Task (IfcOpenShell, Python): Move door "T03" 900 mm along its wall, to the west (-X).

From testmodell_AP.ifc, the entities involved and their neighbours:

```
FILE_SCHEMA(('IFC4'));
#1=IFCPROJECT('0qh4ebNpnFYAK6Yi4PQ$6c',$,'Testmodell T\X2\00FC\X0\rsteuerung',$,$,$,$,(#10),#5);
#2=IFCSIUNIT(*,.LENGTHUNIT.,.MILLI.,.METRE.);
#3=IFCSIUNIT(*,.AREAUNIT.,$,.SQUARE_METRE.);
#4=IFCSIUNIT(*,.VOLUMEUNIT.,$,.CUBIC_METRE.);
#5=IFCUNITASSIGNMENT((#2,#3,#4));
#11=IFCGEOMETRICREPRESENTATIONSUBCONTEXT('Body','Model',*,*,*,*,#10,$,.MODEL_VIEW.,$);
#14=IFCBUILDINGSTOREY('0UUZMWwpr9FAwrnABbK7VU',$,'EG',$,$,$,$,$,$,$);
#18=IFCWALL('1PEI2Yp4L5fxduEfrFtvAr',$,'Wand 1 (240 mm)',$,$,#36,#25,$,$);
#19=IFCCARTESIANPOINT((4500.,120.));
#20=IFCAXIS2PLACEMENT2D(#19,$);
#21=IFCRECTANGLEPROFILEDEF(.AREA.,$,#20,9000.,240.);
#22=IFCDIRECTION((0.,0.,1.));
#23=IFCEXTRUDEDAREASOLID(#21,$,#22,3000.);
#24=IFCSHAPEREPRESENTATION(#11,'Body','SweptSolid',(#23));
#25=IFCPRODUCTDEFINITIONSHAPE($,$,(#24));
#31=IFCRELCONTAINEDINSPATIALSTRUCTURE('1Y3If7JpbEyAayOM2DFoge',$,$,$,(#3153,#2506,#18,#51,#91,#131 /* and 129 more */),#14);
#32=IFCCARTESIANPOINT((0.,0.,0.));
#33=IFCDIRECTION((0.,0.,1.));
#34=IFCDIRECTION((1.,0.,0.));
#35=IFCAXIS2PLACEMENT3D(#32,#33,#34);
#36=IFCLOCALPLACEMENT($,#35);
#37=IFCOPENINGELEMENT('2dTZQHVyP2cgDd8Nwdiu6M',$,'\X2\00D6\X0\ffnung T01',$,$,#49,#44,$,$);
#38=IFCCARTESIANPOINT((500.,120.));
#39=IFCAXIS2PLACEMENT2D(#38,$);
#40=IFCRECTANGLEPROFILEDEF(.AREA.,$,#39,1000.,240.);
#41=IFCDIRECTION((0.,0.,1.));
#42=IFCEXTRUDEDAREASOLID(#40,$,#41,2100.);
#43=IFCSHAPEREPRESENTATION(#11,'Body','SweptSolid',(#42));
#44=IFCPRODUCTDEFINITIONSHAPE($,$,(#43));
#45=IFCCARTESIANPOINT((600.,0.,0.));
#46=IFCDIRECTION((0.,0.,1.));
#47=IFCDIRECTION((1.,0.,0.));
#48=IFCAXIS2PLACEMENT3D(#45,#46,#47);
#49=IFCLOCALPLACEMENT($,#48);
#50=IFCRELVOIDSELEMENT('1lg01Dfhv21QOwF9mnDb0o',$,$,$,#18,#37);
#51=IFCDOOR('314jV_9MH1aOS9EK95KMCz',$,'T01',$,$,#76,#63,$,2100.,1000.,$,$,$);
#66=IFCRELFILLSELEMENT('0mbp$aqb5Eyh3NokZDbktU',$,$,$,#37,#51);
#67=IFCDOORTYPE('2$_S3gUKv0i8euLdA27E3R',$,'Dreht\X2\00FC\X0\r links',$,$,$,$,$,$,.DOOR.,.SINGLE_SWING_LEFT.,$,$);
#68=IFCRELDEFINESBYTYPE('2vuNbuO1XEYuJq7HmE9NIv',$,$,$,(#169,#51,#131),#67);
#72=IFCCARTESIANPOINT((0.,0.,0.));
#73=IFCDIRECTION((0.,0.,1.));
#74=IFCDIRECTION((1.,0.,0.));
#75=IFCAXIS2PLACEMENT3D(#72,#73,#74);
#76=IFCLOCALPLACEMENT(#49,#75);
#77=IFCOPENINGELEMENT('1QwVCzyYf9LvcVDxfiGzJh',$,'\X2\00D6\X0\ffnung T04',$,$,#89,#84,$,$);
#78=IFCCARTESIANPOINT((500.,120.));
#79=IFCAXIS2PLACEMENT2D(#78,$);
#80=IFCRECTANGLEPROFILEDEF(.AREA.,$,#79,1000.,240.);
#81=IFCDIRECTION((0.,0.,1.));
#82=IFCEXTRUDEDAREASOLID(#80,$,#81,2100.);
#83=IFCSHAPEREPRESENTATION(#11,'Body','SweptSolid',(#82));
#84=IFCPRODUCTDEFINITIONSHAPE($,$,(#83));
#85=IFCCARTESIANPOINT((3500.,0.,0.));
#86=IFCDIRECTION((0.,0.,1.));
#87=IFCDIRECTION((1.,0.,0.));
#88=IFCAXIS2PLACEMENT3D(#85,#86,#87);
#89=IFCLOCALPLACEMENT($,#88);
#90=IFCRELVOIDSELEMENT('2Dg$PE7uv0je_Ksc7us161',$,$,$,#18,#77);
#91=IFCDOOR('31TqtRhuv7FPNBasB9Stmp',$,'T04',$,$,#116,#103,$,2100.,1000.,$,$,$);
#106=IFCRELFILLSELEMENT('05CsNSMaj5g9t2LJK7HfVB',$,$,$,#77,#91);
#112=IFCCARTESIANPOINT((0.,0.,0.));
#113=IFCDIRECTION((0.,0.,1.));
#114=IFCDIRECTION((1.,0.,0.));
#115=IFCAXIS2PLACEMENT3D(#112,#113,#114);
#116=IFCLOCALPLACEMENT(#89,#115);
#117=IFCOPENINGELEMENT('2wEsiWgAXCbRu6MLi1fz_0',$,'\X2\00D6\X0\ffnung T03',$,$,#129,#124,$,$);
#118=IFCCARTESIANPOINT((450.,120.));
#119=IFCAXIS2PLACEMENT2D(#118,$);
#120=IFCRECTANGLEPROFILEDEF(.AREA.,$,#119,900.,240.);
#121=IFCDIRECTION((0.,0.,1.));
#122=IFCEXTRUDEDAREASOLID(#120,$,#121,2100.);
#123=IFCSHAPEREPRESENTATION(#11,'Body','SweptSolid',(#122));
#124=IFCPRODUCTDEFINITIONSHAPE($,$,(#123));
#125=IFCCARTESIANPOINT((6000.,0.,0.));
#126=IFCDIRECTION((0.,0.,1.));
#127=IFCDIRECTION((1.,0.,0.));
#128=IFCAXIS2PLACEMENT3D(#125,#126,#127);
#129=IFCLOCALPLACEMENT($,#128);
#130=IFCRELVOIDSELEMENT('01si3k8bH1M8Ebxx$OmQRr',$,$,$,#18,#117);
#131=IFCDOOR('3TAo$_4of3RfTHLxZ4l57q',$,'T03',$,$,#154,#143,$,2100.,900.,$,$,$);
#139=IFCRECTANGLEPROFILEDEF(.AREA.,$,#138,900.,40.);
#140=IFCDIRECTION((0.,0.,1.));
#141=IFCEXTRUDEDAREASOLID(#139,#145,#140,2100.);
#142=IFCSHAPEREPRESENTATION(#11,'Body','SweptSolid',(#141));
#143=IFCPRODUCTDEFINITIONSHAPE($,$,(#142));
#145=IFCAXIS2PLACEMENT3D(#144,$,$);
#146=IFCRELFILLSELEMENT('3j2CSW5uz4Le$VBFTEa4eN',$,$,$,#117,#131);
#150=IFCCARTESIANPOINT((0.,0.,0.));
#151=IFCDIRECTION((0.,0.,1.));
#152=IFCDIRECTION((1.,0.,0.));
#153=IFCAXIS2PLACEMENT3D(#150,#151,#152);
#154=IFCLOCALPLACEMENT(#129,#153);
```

```python
import ifcopenshell
import ifcopenshell.api.geometry
import ifcopenshell.util.placement
import ifcopenshell.util.unit

model = ifcopenshell.open("testmodell_AP.ifc")
unit_scale = ifcopenshell.util.unit.calculate_unit_scale(model)

door = model.by_id(131)
opening = door.FillsVoids[0].RelatingOpeningElement
wall = opening.VoidsElements[0].RelatingBuildingElement

wall_matrix = ifcopenshell.util.placement.get_local_placement(wall.ObjectPlacement)
shift = wall_matrix[:3, 0] * -0.9 / unit_scale
before = ifcopenshell.util.placement.get_local_placement(door.ObjectPlacement)[:3, 3].copy()

# The door is placed relative to its opening, so it follows when the opening moves.
matrix = ifcopenshell.util.placement.get_local_placement(opening.ObjectPlacement)
matrix[:3, 3] += shift
ifcopenshell.api.geometry.edit_object_placement(
    model, product=opening, matrix=matrix, is_si=False, should_transform_children=True
)

after = ifcopenshell.util.placement.get_local_placement(door.ObjectPlacement)[:3, 3]
print("door moved by", (after - before).round(3) + 0.0)

model.write("testmodell_AP_v2.ifc")
```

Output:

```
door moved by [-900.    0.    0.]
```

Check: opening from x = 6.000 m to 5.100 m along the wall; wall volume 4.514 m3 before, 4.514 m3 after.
